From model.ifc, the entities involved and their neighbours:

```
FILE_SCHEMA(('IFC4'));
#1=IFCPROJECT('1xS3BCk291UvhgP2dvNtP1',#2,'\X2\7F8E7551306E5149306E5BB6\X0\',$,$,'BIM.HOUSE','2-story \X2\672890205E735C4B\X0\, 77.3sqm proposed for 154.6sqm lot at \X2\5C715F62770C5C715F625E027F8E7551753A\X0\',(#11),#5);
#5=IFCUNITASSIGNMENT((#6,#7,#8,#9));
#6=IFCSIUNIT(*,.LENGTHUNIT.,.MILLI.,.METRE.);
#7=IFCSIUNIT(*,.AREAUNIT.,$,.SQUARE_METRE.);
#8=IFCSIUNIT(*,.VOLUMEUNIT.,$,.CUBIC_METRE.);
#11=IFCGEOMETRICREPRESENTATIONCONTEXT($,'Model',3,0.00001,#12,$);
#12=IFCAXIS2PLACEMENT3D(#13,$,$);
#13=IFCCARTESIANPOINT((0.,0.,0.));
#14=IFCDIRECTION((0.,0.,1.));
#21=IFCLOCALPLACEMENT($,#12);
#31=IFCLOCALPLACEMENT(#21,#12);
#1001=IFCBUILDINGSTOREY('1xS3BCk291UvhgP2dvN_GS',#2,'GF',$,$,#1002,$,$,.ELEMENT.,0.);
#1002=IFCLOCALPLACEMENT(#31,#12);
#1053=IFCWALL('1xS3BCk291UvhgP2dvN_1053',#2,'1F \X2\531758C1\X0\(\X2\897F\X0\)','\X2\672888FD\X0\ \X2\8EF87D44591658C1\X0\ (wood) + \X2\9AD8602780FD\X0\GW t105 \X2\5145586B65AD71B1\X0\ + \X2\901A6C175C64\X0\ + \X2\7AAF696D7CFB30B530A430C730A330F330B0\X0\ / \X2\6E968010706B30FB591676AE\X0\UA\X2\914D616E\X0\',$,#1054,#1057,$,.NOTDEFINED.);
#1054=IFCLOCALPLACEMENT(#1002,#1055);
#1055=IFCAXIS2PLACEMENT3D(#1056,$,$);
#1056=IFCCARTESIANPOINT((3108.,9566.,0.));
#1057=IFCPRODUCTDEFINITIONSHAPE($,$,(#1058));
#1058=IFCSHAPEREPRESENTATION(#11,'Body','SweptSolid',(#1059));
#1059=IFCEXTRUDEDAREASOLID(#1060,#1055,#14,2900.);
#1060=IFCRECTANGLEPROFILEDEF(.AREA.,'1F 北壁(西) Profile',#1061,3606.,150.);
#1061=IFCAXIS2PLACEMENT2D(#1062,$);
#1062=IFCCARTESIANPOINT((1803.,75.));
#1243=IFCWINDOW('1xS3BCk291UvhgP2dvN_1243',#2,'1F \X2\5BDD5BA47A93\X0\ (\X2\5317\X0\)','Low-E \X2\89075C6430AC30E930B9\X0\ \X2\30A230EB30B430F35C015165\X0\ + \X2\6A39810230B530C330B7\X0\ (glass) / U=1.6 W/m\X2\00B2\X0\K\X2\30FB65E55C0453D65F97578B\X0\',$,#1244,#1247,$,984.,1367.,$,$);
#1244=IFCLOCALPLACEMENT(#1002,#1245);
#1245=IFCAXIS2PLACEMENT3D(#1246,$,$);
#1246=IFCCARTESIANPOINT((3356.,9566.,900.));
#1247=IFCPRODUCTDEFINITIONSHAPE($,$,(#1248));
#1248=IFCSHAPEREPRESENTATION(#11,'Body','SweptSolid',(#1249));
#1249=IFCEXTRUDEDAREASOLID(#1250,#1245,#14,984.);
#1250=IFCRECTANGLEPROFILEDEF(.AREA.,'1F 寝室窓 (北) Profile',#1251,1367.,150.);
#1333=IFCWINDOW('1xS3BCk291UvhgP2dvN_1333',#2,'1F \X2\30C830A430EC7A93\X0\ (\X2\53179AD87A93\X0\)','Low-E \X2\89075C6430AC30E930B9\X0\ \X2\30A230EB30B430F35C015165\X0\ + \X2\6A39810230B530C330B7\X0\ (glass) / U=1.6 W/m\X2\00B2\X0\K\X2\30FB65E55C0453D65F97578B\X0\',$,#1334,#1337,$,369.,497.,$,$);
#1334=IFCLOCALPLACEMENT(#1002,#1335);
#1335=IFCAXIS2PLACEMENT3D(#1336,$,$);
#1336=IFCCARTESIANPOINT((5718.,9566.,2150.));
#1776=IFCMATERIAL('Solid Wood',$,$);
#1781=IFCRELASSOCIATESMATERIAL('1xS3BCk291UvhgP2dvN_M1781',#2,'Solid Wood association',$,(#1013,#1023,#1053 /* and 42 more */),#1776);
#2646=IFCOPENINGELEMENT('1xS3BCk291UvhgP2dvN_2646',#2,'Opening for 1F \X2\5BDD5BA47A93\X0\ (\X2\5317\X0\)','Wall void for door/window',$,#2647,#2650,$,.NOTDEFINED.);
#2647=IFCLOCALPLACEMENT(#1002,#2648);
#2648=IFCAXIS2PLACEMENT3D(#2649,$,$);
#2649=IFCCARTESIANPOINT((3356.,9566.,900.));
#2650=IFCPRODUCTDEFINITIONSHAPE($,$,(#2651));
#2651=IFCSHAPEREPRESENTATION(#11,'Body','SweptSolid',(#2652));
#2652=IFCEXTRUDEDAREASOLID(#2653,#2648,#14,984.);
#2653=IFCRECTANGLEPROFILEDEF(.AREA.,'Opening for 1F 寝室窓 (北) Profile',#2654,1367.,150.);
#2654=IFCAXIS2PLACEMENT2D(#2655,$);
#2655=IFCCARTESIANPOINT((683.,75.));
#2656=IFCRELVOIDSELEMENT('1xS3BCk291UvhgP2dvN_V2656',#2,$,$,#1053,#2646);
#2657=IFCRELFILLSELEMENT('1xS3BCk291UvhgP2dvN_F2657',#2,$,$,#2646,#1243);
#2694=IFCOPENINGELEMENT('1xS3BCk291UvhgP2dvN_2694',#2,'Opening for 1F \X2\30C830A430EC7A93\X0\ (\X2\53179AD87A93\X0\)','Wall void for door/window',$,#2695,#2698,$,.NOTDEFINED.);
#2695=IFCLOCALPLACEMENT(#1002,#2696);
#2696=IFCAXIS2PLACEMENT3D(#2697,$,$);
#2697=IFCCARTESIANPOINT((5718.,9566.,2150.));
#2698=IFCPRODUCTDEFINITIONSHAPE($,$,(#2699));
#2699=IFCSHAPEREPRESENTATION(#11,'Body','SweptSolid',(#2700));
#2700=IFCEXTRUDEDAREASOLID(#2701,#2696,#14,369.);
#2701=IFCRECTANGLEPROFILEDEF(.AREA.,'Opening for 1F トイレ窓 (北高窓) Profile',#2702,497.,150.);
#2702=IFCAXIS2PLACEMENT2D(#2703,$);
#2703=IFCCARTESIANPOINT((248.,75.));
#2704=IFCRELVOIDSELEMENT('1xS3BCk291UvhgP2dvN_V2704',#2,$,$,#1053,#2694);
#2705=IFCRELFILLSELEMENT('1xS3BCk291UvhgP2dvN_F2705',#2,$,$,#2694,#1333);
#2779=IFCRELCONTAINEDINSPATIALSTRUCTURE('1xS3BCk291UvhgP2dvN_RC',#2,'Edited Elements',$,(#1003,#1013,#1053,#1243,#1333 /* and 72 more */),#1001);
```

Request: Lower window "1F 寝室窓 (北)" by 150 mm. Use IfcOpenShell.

```python
import numpy as np
import ifcopenshell
import ifcopenshell.api.geometry
import ifcopenshell.util.placement
import ifcopenshell.util.unit

model = ifcopenshell.open("model.ifc")
unit_scale = ifcopenshell.util.unit.calculate_unit_scale(model)

window = model.by_id(1243)
opening = window.FillsVoids[0].RelatingOpeningElement
dz = -150.0

shift = np.array([0.0, 0.0, dz])
# The window is not placed relative to its opening, so move both.
for product in (opening, window):
    matrix = ifcopenshell.util.placement.get_local_placement(product.ObjectPlacement)
    matrix[:3, 3] += shift
    ifcopenshell.api.geometry.edit_object_placement(model, product=product, matrix=matrix, is_si=False)

print(f"moved by {dz * unit_scale:+.3f} m")

model.write("model_edited.ifc")
```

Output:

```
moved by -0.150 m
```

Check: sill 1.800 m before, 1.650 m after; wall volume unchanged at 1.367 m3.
